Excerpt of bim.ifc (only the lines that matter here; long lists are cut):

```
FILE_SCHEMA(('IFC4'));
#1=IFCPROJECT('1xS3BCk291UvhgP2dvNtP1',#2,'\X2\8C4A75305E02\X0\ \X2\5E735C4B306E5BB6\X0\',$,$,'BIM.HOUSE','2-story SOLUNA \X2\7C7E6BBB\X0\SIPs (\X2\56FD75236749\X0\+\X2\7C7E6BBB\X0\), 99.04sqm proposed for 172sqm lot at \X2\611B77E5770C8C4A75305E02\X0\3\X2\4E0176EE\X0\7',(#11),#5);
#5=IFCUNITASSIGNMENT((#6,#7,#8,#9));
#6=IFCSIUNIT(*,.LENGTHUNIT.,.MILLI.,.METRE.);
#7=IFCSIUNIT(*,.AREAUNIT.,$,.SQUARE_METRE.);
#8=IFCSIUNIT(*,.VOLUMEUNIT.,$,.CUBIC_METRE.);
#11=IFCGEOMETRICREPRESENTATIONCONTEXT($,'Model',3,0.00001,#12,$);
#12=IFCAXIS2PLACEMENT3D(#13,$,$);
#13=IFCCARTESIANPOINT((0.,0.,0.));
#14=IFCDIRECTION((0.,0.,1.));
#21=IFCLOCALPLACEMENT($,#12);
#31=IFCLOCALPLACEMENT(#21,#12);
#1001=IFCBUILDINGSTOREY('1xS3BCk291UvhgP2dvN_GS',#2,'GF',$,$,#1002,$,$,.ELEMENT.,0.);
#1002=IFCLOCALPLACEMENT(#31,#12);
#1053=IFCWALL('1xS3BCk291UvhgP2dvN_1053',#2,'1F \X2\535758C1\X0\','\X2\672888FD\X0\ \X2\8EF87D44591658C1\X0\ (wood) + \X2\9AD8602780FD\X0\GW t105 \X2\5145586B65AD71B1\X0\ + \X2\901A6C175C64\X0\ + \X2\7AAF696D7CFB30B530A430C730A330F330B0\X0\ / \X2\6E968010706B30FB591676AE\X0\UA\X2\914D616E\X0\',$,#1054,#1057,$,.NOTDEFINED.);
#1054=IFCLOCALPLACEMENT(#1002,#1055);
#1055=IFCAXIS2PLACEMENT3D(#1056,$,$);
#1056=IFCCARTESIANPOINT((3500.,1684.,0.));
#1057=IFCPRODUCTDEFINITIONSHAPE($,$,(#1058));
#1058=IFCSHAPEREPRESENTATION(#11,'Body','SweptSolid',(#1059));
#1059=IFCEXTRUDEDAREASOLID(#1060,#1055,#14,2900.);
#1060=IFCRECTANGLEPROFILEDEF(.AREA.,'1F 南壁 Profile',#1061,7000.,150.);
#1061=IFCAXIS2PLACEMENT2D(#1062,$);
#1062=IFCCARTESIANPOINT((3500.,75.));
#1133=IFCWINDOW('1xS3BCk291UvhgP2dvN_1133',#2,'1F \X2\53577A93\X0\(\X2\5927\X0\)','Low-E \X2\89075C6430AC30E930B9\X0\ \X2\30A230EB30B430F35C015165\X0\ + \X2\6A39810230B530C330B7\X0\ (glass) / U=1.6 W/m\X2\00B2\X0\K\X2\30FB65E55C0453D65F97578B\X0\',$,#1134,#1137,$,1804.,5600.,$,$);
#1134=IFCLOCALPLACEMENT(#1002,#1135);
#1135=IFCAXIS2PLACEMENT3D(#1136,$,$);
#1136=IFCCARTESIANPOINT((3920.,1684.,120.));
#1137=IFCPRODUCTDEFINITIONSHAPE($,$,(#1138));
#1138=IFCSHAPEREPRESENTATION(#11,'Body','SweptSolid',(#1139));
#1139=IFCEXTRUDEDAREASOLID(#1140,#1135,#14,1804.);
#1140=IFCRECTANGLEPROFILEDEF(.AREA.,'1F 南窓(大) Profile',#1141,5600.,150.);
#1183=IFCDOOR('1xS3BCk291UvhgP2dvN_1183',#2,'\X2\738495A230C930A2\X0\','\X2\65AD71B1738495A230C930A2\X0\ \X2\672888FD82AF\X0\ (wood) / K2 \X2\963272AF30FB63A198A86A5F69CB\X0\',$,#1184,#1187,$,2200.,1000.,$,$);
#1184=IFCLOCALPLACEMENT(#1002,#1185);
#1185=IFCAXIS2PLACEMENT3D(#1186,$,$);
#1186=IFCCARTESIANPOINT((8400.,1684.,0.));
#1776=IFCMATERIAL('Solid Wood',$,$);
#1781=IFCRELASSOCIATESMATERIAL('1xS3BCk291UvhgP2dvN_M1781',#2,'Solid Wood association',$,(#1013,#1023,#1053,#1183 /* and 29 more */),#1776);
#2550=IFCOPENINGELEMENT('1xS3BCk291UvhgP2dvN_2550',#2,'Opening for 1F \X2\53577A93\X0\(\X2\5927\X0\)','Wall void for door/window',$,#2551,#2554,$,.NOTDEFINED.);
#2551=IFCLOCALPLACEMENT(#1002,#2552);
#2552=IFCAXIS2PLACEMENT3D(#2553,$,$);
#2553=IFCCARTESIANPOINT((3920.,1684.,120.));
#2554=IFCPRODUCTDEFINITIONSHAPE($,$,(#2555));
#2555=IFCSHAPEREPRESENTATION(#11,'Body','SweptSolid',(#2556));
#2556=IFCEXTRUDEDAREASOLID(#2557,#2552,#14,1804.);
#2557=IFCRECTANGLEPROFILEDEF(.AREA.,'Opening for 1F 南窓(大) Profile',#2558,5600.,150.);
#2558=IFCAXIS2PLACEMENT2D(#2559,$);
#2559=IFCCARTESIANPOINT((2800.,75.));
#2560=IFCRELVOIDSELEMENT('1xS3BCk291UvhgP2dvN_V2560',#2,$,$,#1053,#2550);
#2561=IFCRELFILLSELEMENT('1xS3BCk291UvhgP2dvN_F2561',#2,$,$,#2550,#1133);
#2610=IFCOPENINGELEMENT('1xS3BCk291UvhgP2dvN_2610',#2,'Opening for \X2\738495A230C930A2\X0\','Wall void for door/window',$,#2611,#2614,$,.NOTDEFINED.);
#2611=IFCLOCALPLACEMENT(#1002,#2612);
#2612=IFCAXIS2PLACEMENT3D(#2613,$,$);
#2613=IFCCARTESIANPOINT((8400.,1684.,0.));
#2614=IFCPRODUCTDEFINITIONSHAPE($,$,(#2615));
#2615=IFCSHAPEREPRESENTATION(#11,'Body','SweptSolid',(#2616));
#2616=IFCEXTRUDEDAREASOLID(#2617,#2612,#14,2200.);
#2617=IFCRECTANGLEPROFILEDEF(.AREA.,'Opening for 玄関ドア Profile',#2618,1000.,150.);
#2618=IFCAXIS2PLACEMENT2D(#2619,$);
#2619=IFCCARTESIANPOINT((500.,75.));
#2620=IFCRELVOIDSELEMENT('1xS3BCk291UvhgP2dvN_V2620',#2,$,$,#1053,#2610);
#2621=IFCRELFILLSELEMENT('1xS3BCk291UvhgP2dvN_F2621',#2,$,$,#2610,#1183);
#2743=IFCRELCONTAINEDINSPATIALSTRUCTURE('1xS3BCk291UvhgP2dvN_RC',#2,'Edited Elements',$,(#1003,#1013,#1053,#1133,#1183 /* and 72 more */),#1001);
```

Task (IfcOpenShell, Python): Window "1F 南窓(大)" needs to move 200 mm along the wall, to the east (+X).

```python
import ifcopenshell
import ifcopenshell.api.geometry
import ifcopenshell.util.placement

model = ifcopenshell.open("bim.ifc")

window = model.by_id(1133)
opening = window.FillsVoids[0].RelatingOpeningElement
wall = opening.VoidsElements[0].RelatingBuildingElement

wall_matrix = ifcopenshell.util.placement.get_local_placement(wall.ObjectPlacement)
shift = wall_matrix[:3, 0] * 200.0
before = ifcopenshell.util.placement.get_local_placement(window.ObjectPlacement)[:3, 3].copy()

# The window is not placed relative to its opening, so move both.
for product in (opening, window):
    matrix = ifcopenshell.util.placement.get_local_placement(product.ObjectPlacement)
    matrix[:3, 3] += shift
    ifcopenshell.api.geometry.edit_object_placement(model, product=product, matrix=matrix, is_si=False)

after = ifcopenshell.util.placement.get_local_placement(window.ObjectPlacement)[:3, 3]
print("window moved by", (after - before).round(3) + 0.0)

model.write("bim-out.ifc")
```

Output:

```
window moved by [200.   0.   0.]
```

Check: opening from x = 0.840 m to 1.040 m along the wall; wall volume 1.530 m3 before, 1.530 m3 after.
